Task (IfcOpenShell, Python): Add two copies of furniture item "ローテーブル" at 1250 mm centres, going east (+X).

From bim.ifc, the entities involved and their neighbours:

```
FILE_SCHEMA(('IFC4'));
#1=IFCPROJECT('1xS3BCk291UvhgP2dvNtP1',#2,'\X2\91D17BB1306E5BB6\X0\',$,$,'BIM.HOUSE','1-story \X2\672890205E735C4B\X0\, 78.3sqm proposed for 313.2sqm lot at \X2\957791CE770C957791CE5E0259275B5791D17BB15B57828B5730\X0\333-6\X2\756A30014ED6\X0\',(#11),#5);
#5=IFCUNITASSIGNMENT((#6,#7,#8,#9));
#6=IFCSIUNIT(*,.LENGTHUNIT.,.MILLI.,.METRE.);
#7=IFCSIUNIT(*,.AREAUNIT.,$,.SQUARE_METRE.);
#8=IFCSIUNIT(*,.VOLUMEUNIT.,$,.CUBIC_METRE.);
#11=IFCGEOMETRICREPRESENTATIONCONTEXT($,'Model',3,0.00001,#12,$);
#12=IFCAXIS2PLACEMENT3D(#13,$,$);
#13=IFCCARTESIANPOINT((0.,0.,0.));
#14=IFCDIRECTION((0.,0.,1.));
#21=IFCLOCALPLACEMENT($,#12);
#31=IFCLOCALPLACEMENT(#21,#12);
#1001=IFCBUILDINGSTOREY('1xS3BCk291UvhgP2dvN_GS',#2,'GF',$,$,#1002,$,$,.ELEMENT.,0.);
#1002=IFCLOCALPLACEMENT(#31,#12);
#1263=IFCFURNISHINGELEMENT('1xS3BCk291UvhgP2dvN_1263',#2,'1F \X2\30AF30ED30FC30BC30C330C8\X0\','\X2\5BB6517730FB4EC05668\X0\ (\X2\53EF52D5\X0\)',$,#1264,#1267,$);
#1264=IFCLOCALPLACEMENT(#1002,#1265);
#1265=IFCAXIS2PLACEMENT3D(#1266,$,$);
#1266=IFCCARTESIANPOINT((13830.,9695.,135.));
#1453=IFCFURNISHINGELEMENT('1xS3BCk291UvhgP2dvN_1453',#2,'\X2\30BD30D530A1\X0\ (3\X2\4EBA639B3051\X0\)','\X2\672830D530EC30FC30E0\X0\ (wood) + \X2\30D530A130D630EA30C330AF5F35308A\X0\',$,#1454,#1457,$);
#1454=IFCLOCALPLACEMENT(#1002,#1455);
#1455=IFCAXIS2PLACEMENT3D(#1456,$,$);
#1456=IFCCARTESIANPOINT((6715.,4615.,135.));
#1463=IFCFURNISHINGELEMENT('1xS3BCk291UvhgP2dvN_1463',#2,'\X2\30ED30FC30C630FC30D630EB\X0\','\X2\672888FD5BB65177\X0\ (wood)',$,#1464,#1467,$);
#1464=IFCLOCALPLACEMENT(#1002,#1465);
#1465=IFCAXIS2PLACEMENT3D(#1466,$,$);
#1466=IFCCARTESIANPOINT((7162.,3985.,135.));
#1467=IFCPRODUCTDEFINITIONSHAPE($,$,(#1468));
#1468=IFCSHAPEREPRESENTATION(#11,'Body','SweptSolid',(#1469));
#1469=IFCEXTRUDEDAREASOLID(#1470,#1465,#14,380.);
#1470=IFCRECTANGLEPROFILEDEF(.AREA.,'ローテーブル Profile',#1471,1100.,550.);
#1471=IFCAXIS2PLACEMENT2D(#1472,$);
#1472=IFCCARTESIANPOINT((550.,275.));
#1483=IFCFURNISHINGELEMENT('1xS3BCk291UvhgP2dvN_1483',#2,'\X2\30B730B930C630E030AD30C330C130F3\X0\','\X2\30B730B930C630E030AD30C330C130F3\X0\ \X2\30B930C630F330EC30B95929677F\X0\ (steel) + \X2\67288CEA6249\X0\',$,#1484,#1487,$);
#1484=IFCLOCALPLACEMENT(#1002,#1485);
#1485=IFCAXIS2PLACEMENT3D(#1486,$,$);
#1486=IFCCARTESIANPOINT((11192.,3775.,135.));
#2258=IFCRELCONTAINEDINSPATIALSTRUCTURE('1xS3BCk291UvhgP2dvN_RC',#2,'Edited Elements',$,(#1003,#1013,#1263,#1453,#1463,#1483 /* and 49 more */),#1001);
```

```python
import numpy as np
import ifcopenshell
import ifcopenshell.api.geometry
import ifcopenshell.api.root
import ifcopenshell.util.element
import ifcopenshell.util.placement

model = ifcopenshell.open("bim.ifc")


def reuse_history(source, copy):
    """copy_class also copies each property set's owner history, people and application; keep the originals."""
    for rel in copy.IsDefinedBy:
        if rel.is_a("IfcRelDefinesByProperties") and (history := rel.RelatingPropertyDefinition.OwnerHistory):
            rel.RelatingPropertyDefinition.OwnerHistory = source.OwnerHistory
            ifcopenshell.util.element.remove_deep2(model, history)


source = model.by_id(1463)
base = ifcopenshell.util.placement.get_local_placement(source.ObjectPlacement)
step = np.array([1.0, 0.0, 0.0]) * 1250.0

for i in range(1, 3):
    copy = ifcopenshell.api.root.copy_class(model, product=source)
    copy.Representation = ifcopenshell.util.element.copy_deep(
        model, source.Representation, exclude=["IfcGeometricRepresentationContext", "IfcRepresentationMap"]
    )
    reuse_history(source, copy)
    matrix = base.copy()
    matrix[:3, 3] += i * step
    print("added at", matrix[:3, 3].round(3) + 0.0)
    ifcopenshell.api.geometry.edit_object_placement(model, product=copy, matrix=matrix, is_si=False)

model.write("bim-out.ifc")
```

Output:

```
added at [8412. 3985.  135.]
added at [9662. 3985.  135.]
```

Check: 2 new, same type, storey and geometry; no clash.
